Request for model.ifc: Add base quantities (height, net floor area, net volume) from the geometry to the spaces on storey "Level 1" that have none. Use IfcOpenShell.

First a look at what the model holds.

```python
import ifcopenshell
import ifcopenshell.util.element
import ifcopenshell.util.unit

model = ifcopenshell.open("model.ifc")
print(model.schema)
for unit_type in ("LENGTHUNIT", "AREAUNIT", "VOLUMEUNIT"):
    print(unit_type, ifcopenshell.util.unit.calculate_unit_scale(model, unit_type))
storey = next(s for s in model.by_type("IfcBuildingStorey") if s.Name == "Level 1")
spaces = [e for e in ifcopenshell.util.element.get_decomposition(storey) if e.is_a("IfcSpace")]
for e in sorted(spaces, key=lambda e: e.id()):
    print(e.id(), e.is_a(), e.Name, list(ifcopenshell.util.element.get_psets(e, qtos_only=True)), sep=" | ")
```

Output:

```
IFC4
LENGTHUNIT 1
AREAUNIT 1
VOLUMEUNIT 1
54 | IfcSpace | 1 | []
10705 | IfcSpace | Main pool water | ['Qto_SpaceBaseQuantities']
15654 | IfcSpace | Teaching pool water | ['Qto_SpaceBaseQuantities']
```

```python
import ifcopenshell
import ifcopenshell.api.pset
import ifcopenshell.geom
import ifcopenshell.util.element
import ifcopenshell.util.shape
import ifcopenshell.util.unit

model = ifcopenshell.open("model.ifc")
unit_scale = ifcopenshell.util.unit.calculate_unit_scale(model)
area_scale = ifcopenshell.util.unit.calculate_unit_scale(model, "AREAUNIT")
volume_scale = ifcopenshell.util.unit.calculate_unit_scale(model, "VOLUMEUNIT")
settings = ifcopenshell.geom.settings()

storey = next(s for s in model.by_type("IfcBuildingStorey") if s.Name == "Level 1")
spaces = [e for e in ifcopenshell.util.element.get_decomposition(storey) if e.is_a("IfcSpace")]

for e in sorted(spaces, key=lambda e: e.id()):
    if ifcopenshell.util.element.get_psets(e, qtos_only=True, should_inherit=False):
        continue
    # Geometry comes back in metres, in the element's own axes.
    shape = ifcopenshell.geom.create_shape(settings, e)
    values = {
        "Height": ifcopenshell.util.shape.get_z(shape.geometry) / unit_scale,
        "NetFloorArea": ifcopenshell.util.shape.get_footprint_area(shape.geometry) / area_scale,
        "NetVolume": ifcopenshell.util.shape.get_volume(shape.geometry) / volume_scale,
    }
    qto = ifcopenshell.api.pset.add_qto(model, product=e, name="Qto_SpaceBaseQuantities")
    ifcopenshell.api.pset.edit_qto(model, qto=qto, properties=values)
    print(e.id(), {k: round(v, 3) for k, v in values.items()})

model.write("model_edited.ifc")
```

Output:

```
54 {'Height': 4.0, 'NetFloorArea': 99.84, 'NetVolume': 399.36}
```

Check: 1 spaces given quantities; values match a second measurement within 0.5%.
